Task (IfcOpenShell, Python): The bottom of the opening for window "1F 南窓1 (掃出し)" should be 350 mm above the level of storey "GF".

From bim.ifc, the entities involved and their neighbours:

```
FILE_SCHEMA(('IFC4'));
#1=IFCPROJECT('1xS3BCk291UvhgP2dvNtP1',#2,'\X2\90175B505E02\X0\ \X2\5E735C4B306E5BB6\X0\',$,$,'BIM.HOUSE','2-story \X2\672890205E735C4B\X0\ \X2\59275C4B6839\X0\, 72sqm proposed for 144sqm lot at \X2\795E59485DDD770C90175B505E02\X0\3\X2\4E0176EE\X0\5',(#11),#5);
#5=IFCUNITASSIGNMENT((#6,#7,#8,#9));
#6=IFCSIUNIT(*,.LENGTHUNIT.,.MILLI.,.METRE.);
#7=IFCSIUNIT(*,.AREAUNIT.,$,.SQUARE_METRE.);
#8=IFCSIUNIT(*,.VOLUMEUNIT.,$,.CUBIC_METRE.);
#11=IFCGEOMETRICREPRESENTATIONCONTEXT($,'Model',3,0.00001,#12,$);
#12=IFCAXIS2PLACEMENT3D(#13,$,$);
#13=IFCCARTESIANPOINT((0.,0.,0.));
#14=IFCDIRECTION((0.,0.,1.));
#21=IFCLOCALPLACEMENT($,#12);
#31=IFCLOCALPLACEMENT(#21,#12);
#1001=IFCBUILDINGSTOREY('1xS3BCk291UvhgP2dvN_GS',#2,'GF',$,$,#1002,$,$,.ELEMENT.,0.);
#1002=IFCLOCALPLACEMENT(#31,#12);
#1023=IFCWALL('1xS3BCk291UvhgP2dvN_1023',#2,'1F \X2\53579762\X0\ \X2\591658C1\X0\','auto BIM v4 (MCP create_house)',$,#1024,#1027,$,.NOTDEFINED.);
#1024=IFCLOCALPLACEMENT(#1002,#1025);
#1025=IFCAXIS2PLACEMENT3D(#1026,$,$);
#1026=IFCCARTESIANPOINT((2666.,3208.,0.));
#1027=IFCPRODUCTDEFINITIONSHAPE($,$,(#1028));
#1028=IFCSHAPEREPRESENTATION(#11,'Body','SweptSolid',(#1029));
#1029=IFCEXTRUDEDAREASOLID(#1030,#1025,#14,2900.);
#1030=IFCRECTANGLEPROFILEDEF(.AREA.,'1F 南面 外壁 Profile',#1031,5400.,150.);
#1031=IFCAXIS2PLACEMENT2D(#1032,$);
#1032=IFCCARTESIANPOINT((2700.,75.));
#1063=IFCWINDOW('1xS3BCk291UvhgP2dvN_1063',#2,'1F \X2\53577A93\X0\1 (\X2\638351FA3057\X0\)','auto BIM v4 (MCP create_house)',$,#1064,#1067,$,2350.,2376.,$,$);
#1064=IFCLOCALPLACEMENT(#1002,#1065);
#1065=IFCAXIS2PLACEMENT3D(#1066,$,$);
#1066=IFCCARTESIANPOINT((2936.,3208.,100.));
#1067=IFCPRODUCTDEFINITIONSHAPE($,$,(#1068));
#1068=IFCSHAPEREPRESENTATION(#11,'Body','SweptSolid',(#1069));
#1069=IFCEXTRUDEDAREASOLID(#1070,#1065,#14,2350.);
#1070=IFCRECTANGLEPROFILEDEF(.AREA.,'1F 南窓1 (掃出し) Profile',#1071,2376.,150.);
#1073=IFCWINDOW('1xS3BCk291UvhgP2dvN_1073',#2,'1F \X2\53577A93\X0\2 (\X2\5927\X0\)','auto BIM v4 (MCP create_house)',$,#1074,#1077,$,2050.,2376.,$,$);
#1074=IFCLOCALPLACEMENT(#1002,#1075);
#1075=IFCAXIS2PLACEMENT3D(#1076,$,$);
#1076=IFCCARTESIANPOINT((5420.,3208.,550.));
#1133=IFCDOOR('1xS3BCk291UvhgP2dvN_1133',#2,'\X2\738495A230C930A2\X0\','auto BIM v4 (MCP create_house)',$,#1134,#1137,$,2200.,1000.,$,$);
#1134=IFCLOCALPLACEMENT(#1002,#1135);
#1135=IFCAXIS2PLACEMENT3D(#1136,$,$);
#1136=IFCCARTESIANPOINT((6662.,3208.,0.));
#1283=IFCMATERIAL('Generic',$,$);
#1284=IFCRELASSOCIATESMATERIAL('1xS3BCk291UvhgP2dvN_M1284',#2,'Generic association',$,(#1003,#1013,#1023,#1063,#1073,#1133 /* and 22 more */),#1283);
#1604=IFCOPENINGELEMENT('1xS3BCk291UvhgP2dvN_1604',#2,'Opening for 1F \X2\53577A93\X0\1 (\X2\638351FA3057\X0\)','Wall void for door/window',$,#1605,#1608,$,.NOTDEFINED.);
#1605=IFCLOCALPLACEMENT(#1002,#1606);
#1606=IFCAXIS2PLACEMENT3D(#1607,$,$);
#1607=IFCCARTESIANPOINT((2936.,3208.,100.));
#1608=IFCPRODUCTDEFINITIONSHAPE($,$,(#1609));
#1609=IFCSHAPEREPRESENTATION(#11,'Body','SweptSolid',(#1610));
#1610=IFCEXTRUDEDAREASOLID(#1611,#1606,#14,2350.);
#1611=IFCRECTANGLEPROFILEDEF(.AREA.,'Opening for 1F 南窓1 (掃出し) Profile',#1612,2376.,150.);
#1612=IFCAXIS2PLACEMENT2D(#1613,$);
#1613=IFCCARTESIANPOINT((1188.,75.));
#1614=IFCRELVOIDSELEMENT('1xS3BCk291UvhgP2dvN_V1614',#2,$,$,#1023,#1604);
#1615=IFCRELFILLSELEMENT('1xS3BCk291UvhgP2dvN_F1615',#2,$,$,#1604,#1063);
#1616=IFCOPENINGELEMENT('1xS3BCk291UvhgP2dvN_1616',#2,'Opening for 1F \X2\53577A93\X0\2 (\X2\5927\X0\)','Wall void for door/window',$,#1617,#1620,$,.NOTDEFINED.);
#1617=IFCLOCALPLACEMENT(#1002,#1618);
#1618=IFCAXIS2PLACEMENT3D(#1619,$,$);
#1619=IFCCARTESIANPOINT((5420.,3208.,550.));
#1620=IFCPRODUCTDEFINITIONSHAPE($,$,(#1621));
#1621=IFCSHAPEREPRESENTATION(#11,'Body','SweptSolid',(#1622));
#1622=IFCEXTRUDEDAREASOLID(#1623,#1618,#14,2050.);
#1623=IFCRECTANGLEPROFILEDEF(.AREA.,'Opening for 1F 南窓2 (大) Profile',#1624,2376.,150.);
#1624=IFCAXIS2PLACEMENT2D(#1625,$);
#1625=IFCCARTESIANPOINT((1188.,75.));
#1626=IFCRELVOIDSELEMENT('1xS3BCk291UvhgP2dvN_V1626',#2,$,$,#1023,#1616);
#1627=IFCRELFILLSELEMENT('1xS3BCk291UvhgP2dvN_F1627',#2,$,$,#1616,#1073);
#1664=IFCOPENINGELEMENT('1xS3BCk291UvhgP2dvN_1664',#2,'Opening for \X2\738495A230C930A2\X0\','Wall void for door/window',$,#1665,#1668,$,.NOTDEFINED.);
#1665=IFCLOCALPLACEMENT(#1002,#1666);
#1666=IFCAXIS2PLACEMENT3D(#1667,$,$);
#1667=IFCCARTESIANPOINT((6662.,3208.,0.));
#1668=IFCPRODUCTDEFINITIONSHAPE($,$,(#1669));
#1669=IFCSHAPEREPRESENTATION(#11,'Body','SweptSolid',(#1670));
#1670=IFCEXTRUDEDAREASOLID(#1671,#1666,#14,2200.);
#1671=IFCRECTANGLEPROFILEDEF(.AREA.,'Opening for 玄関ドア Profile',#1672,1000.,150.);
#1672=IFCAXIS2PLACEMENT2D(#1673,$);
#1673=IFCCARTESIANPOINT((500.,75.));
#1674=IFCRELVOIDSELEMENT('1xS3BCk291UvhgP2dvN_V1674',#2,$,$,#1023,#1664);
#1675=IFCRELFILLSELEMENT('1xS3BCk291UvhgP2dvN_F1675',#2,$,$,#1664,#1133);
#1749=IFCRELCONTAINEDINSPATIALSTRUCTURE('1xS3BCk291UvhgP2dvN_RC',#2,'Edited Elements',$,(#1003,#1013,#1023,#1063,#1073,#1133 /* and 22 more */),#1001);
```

```python
import numpy as np
import ifcopenshell
import ifcopenshell.api.geometry
import ifcopenshell.geom
import ifcopenshell.util.element
import ifcopenshell.util.placement
import ifcopenshell.util.shape
import ifcopenshell.util.unit

model = ifcopenshell.open("bim.ifc")
unit_scale = ifcopenshell.util.unit.calculate_unit_scale(model)

window = model.by_id(1063)
opening = window.FillsVoids[0].RelatingOpeningElement
storey = ifcopenshell.util.element.get_container(window, ifc_class="IfcBuildingStorey")
level = ifcopenshell.util.placement.get_local_placement(storey.ObjectPlacement)[2, 3]

# The opening's origin need not be at the sill, so measure its lowest point.
shape = ifcopenshell.geom.create_shape(ifcopenshell.geom.settings(), opening)
bottom = ifcopenshell.util.shape.get_shape_bottom_elevation(shape, shape.geometry) / unit_scale
dz = level + 350.0 - bottom

shift = np.array([0.0, 0.0, dz])
# The window is not placed relative to its opening, so move both.
for product in (opening, window):
    matrix = ifcopenshell.util.placement.get_local_placement(product.ObjectPlacement)
    matrix[:3, 3] += shift
    ifcopenshell.api.geometry.edit_object_placement(model, product=product, matrix=matrix, is_si=False)

print(f"moved by {dz * unit_scale:+.3f} m")

model.write("bim_v2.ifc")
```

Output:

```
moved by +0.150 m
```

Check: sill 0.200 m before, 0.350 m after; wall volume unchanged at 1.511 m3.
